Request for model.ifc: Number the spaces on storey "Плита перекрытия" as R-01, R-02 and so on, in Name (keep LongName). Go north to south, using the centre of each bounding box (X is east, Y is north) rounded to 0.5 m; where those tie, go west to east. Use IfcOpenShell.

First a look at what the model holds.

```python
import ifcopenshell
import ifcopenshell.util.element
import ifcopenshell.util.placement

model = ifcopenshell.open("model.ifc")
print(model.schema)
storey = next(s for s in model.by_type("IfcBuildingStorey") if s.Name == "Плита перекрытия")
spaces = [e for e in ifcopenshell.util.element.get_decomposition(storey) if e.is_a("IfcSpace")]
for e in sorted(spaces, key=lambda e: e.id()):
    origin = ifcopenshell.util.placement.get_local_placement(e.ObjectPlacement)[:3, 3]
    print(e.id(), e.Name, e.LongName, origin.round(2) + 0.0, sep=" | ")
```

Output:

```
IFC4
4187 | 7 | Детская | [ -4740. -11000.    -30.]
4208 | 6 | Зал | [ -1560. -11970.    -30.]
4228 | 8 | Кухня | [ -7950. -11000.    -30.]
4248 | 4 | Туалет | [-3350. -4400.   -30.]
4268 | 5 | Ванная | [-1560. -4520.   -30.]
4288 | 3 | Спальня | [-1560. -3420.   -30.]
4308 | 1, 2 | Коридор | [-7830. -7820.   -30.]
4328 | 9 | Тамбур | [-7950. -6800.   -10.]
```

```python
import ifcopenshell
import ifcopenshell.geom
import ifcopenshell.util.element
import ifcopenshell.util.shape

model = ifcopenshell.open("model.ifc")
settings = ifcopenshell.geom.settings()
settings.set("use-world-coords", True)


def centre(element):
    shape = ifcopenshell.geom.create_shape(settings, element)
    return ifcopenshell.util.shape.get_bbox_centroid(shape.geometry)


storey = next(s for s in model.by_type("IfcBuildingStorey") if s.Name == "Плита перекрытия")
spaces = [e for e in ifcopenshell.util.element.get_decomposition(storey) if e.is_a("IfcSpace")]

# Insertion points can sit at a corner or the storey origin, so sort by the geometry (in metres).
centres = {e: centre(e) for e in spaces}
spaces.sort(key=lambda e: (-round(centres[e][1] / 0.5), centres[e][0]))

for i, e in enumerate(spaces, start=1):
    number = f"R-{i:02d}"
    e.Name = number
    print(e.id(), number)

model.write("model-out.ifc")
```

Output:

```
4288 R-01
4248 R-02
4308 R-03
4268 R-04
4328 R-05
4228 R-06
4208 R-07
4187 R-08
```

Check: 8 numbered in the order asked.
